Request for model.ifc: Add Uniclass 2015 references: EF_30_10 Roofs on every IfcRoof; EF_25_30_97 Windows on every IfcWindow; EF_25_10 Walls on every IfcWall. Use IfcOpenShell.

First a look at what the model holds.

```python
import ifcopenshell

model = ifcopenshell.open("model.ifc")
print(model.schema)
print("classifications:", [c.Name for c in model.by_type("IfcClassification")])
for ifc_class in ("IfcDoor", "IfcRoof", "IfcStair", "IfcWall", "IfcWindow"):
    print(ifc_class, len(model.by_type(ifc_class)))
```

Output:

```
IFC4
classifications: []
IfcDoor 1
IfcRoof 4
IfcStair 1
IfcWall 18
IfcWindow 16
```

```python
import ifcopenshell
import ifcopenshell.api.classification

model = ifcopenshell.open("model.ifc")

system = ifcopenshell.api.classification.add_classification(model, classification="Uniclass 2015")

codes = {
    "IfcRoof": ("EF_30_10", "Roofs"),
    "IfcWindow": ("EF_25_30_97", "Windows"),
    "IfcWall": ("EF_25_10", "Walls"),
}
for ifc_class, (code, name) in codes.items():
    products = model.by_type(ifc_class)
    ifcopenshell.api.classification.add_reference(
        model, products=products, classification=system, identification=code, name=name
    )
    print(code, len(products))

model.write("model_rev.ifc")
```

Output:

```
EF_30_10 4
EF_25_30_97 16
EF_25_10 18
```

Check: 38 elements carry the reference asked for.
